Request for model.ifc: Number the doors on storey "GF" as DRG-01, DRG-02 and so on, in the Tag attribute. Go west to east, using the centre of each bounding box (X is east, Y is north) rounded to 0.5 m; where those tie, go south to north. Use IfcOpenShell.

First a look at what the model holds.

```python
import ifcopenshell
import ifcopenshell.util.element
import ifcopenshell.util.placement

model = ifcopenshell.open("model.ifc")
print(model.schema)
storey = next(s for s in model.by_type("IfcBuildingStorey") if s.Name == "GF")
doors = [e for e in ifcopenshell.util.element.get_decomposition(storey) if e.is_a("IfcDoor")]
for e in sorted(doors, key=lambda e: e.id()):
    origin = ifcopenshell.util.placement.get_local_placement(e.ObjectPlacement)[:3, 3]
    print(e.id(), e.Tag, e.Name, origin.round(2) + 0.0, sep=" | ")
```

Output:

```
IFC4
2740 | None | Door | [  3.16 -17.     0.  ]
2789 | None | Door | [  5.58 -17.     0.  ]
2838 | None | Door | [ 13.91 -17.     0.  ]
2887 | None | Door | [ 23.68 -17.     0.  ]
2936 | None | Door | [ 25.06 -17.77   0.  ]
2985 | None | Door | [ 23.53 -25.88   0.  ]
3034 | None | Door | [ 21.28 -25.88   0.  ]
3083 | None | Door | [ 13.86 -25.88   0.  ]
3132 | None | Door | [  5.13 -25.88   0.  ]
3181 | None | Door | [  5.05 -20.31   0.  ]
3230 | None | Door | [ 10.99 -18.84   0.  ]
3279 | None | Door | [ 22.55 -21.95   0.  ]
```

```python
import ifcopenshell
import ifcopenshell.geom
import ifcopenshell.util.element
import ifcopenshell.util.shape

model = ifcopenshell.open("model.ifc")
settings = ifcopenshell.geom.settings()
settings.set("use-world-coords", True)


def centre(element):
    shape = ifcopenshell.geom.create_shape(settings, element)
    return ifcopenshell.util.shape.get_bbox_centroid(shape.geometry)


storey = next(s for s in model.by_type("IfcBuildingStorey") if s.Name == "GF")
doors = [e for e in ifcopenshell.util.element.get_decomposition(storey) if e.is_a("IfcDoor")]

# Insertion points can sit at a corner or the storey origin, so sort by the geometry (in metres).
centres = {e: centre(e) for e in doors}
doors.sort(key=lambda e: (round(centres[e][0] / 0.5), centres[e][1]))

for i, e in enumerate(doors, start=1):
    number = f"DRG-{i:02d}"
    e.Tag = number
    print(e.id(), number)

model.write("model_v2.ifc")
```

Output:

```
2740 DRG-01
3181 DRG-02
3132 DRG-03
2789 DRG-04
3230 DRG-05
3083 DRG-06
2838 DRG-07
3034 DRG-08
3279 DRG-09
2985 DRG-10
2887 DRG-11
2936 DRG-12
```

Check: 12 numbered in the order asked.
